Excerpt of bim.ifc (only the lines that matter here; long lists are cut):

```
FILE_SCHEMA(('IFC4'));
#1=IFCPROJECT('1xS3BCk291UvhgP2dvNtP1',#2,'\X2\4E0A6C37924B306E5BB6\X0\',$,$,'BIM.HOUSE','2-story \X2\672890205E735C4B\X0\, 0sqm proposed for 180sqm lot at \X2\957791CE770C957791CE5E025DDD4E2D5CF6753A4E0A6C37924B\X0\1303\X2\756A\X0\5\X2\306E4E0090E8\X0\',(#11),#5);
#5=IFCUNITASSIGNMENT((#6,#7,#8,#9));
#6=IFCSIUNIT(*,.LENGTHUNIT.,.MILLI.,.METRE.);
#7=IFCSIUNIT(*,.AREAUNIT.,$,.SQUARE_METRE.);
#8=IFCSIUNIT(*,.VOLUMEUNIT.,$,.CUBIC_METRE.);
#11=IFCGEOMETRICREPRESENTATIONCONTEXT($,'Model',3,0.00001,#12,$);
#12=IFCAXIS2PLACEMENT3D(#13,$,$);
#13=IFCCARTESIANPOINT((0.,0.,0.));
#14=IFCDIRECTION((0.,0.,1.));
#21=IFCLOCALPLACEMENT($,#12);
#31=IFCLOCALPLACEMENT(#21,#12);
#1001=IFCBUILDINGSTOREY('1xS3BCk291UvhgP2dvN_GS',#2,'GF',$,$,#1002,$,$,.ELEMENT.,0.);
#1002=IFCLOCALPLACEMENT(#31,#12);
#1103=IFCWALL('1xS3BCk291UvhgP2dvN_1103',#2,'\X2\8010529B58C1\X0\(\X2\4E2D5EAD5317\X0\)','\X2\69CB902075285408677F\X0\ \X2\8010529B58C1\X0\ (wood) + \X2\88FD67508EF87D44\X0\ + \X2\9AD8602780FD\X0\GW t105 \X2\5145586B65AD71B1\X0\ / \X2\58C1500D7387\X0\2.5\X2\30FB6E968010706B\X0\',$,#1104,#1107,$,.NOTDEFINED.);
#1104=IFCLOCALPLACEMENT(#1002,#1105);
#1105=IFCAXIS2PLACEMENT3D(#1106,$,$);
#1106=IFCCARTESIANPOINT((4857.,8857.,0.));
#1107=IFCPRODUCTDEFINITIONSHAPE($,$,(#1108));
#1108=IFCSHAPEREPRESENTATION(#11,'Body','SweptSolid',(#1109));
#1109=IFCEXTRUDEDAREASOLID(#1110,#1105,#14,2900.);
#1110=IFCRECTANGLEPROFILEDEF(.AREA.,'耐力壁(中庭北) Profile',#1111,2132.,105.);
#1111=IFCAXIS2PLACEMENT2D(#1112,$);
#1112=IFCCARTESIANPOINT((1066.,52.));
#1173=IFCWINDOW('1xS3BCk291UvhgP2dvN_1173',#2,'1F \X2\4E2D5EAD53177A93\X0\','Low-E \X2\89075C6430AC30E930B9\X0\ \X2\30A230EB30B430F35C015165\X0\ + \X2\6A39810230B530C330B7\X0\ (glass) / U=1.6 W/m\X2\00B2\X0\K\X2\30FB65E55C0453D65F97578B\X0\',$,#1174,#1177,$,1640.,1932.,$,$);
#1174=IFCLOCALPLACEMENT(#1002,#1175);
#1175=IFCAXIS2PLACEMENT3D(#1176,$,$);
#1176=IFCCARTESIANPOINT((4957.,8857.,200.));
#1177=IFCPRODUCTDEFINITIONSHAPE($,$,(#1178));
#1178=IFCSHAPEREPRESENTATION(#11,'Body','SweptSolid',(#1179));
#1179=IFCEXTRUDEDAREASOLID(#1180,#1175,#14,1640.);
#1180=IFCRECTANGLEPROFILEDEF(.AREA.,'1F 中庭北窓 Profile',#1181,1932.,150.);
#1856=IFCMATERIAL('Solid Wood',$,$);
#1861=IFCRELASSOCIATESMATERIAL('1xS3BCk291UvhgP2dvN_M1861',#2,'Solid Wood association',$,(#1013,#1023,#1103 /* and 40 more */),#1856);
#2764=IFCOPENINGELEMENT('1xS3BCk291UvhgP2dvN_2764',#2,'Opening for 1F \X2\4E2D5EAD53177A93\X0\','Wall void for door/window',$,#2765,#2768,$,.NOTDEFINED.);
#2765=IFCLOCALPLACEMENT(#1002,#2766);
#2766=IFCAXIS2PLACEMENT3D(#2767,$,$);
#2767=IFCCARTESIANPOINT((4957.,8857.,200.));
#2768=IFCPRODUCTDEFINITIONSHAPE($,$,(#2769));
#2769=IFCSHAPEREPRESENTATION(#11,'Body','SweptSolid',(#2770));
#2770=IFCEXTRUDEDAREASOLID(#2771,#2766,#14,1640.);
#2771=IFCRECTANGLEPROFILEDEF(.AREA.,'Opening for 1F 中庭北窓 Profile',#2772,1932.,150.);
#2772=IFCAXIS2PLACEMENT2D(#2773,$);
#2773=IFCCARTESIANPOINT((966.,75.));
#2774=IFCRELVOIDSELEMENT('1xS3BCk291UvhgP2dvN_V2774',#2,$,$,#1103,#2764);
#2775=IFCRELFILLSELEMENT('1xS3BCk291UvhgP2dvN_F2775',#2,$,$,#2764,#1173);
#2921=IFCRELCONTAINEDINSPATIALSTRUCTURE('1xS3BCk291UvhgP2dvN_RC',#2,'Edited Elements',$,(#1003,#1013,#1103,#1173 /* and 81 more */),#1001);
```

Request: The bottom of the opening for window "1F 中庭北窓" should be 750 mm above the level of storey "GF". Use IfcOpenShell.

```python
import numpy as np
import ifcopenshell
import ifcopenshell.api.geometry
import ifcopenshell.geom
import ifcopenshell.util.element
import ifcopenshell.util.placement
import ifcopenshell.util.shape
import ifcopenshell.util.unit

model = ifcopenshell.open("bim.ifc")
unit_scale = ifcopenshell.util.unit.calculate_unit_scale(model)

window = model.by_guid("1xS3BCk291UvhgP2dvN_1173")
opening = window.FillsVoids[0].RelatingOpeningElement
storey = ifcopenshell.util.element.get_container(window, ifc_class="IfcBuildingStorey")
level = ifcopenshell.util.placement.get_local_placement(storey.ObjectPlacement)[2, 3]

# The opening's origin need not be at the sill, so measure its lowest point.
shape = ifcopenshell.geom.create_shape(ifcopenshell.geom.settings(), opening)
bottom = ifcopenshell.util.shape.get_shape_bottom_elevation(shape, shape.geometry) / unit_scale
dz = level + 0.75 / unit_scale - bottom

shift = np.array([0.0, 0.0, dz])
# The window is not placed relative to its opening, so move both.
for product in (opening, window):
    matrix = ifcopenshell.util.placement.get_local_placement(product.ObjectPlacement)
    matrix[:3, 3] += shift
    ifcopenshell.api.geometry.edit_object_placement(model, product=product, matrix=matrix, is_si=False)

print(f"moved by {dz * unit_scale:+.3f} m")

model.write("bim_v2.ifc")
```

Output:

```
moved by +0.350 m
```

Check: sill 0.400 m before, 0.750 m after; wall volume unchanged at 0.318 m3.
